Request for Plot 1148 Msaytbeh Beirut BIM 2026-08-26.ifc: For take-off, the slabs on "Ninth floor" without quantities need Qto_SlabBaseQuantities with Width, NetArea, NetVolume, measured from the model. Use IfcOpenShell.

First a look at what the model holds.

```python
import ifcopenshell
import ifcopenshell.util.element
import ifcopenshell.util.unit

model = ifcopenshell.open("Plot 1148 Msaytbeh Beirut BIM 2026-08-26.ifc")
print(model.schema)
for unit_type in ("LENGTHUNIT", "AREAUNIT", "VOLUMEUNIT"):
    print(unit_type, ifcopenshell.util.unit.calculate_unit_scale(model, unit_type))
storey = next(s for s in model.by_type("IfcBuildingStorey") if s.Name == "Ninth floor")
slabs = [e for e in ifcopenshell.util.element.get_decomposition(storey) if e.is_a("IfcSlab")]
for e in sorted(slabs, key=lambda e: e.id()):
    print(e.id(), e.is_a(), e.Name, list(ifcopenshell.util.element.get_psets(e, qtos_only=True)), sep=" | ")
```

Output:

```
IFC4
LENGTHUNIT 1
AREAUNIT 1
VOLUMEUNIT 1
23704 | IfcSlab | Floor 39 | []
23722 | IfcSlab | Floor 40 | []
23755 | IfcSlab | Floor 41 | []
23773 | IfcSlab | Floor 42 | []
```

```python
import ifcopenshell
import ifcopenshell.api.pset
import ifcopenshell.geom
import ifcopenshell.util.element
import ifcopenshell.util.shape
import ifcopenshell.util.unit

model = ifcopenshell.open("Plot 1148 Msaytbeh Beirut BIM 2026-08-26.ifc")
unit_scale = ifcopenshell.util.unit.calculate_unit_scale(model)
area_scale = ifcopenshell.util.unit.calculate_unit_scale(model, "AREAUNIT")
volume_scale = ifcopenshell.util.unit.calculate_unit_scale(model, "VOLUMEUNIT")
settings = ifcopenshell.geom.settings()

storey = next(s for s in model.by_type("IfcBuildingStorey") if s.Name == "Ninth floor")
slabs = [e for e in ifcopenshell.util.element.get_decomposition(storey) if e.is_a("IfcSlab")]

for e in sorted(slabs, key=lambda e: e.id()):
    if ifcopenshell.util.element.get_psets(e, qtos_only=True, should_inherit=False):
        continue
    # Geometry comes back in metres, in the element's own axes.
    shape = ifcopenshell.geom.create_shape(settings, e)
    values = {
        "Width": ifcopenshell.util.shape.get_z(shape.geometry) / unit_scale,
        "NetArea": ifcopenshell.util.shape.get_footprint_area(shape.geometry) / area_scale,
        "NetVolume": ifcopenshell.util.shape.get_volume(shape.geometry) / volume_scale,
    }
    qto = ifcopenshell.api.pset.add_qto(model, product=e, name="Qto_SlabBaseQuantities")
    ifcopenshell.api.pset.edit_qto(model, qto=qto, properties=values)
    print(e.id(), {k: round(v, 3) for k, v in values.items()})

model.write("Plot 1148 Msaytbeh Beirut BIM 2026-08-26_v2.ifc")
```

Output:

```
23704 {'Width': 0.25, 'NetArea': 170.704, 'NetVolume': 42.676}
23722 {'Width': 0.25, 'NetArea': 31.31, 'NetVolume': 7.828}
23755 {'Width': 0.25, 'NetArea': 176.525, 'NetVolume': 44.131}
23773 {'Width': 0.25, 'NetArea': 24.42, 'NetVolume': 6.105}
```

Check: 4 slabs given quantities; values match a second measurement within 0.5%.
